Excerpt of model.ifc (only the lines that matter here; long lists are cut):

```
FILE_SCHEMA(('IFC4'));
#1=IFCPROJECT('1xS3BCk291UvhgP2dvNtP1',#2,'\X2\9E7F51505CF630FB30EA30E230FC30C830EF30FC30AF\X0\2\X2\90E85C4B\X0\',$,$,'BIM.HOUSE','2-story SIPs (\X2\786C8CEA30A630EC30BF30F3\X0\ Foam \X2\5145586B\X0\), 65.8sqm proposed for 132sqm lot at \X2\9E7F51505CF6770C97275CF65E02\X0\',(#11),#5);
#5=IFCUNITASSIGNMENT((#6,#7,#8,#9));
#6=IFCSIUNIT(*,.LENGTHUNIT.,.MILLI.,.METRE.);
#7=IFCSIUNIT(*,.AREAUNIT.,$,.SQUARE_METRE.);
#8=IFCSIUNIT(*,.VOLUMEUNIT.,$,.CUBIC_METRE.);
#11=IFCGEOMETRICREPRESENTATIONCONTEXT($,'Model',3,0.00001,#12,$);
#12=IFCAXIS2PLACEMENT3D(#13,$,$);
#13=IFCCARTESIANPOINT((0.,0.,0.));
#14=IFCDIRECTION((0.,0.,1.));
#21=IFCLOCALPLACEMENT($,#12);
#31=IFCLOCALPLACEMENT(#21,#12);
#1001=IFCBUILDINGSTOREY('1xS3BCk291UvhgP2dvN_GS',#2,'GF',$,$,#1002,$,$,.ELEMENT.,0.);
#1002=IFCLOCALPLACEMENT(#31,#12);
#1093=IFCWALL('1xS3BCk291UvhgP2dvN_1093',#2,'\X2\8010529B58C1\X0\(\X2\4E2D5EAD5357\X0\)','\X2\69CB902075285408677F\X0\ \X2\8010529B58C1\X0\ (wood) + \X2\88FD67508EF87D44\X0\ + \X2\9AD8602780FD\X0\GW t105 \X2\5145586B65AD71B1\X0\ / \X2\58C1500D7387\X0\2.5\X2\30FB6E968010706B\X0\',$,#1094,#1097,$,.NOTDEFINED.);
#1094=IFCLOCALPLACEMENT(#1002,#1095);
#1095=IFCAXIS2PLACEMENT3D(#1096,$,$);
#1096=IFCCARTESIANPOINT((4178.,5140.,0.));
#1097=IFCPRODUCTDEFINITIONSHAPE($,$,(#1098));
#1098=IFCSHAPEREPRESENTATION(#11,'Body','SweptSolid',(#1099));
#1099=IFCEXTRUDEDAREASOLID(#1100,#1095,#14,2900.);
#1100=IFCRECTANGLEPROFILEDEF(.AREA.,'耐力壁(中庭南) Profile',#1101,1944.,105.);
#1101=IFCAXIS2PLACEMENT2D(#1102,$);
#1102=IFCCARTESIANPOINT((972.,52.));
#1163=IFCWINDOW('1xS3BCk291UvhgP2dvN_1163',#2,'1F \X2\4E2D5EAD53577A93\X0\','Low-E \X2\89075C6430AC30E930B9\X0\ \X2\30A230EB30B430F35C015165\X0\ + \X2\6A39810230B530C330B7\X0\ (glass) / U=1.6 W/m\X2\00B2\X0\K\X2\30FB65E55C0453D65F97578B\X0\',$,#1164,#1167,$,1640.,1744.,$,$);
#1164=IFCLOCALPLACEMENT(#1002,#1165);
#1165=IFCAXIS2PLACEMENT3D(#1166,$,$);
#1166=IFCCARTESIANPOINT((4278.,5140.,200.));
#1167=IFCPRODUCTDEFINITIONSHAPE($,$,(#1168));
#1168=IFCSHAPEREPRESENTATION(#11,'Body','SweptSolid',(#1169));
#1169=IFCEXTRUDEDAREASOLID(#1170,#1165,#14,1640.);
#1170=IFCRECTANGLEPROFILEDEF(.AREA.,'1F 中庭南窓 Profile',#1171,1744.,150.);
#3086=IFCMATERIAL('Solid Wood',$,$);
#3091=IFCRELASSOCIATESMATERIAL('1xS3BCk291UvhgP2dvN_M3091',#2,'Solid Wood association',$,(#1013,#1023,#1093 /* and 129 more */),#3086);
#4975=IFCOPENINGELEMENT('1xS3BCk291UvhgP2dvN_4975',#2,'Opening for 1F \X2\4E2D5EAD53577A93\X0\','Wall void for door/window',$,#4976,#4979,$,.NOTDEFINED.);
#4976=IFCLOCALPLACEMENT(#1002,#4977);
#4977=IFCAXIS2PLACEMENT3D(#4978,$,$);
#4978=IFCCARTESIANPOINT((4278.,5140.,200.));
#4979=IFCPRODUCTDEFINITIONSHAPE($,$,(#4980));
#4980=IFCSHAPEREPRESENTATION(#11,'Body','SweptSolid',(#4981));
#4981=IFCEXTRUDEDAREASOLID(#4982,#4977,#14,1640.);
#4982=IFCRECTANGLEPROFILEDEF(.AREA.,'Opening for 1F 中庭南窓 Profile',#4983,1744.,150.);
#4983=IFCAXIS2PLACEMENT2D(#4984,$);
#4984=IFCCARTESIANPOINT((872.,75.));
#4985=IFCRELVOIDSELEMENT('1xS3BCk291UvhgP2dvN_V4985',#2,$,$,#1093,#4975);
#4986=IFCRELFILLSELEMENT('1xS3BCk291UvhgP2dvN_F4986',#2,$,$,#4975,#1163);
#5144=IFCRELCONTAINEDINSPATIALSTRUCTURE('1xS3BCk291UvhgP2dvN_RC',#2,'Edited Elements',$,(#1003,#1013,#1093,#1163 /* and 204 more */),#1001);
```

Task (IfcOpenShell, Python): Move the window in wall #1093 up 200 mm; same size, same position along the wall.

```python
import numpy as np
import ifcopenshell
import ifcopenshell.api.geometry
import ifcopenshell.util.placement
import ifcopenshell.util.unit

model = ifcopenshell.open("model.ifc")
unit_scale = ifcopenshell.util.unit.calculate_unit_scale(model)

window = model.by_guid("1xS3BCk291UvhgP2dvN_1163")
opening = window.FillsVoids[0].RelatingOpeningElement
dz = 0.2 / unit_scale

shift = np.array([0.0, 0.0, dz])
# The window is not placed relative to its opening, so move both.
for product in (opening, window):
    matrix = ifcopenshell.util.placement.get_local_placement(product.ObjectPlacement)
    matrix[:3, 3] += shift
    ifcopenshell.api.geometry.edit_object_placement(model, product=product, matrix=matrix, is_si=False)

print(f"moved by {dz * unit_scale:+.3f} m")

model.write("model_v2.ifc")
```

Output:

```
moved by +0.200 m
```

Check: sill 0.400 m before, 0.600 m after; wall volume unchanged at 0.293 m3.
